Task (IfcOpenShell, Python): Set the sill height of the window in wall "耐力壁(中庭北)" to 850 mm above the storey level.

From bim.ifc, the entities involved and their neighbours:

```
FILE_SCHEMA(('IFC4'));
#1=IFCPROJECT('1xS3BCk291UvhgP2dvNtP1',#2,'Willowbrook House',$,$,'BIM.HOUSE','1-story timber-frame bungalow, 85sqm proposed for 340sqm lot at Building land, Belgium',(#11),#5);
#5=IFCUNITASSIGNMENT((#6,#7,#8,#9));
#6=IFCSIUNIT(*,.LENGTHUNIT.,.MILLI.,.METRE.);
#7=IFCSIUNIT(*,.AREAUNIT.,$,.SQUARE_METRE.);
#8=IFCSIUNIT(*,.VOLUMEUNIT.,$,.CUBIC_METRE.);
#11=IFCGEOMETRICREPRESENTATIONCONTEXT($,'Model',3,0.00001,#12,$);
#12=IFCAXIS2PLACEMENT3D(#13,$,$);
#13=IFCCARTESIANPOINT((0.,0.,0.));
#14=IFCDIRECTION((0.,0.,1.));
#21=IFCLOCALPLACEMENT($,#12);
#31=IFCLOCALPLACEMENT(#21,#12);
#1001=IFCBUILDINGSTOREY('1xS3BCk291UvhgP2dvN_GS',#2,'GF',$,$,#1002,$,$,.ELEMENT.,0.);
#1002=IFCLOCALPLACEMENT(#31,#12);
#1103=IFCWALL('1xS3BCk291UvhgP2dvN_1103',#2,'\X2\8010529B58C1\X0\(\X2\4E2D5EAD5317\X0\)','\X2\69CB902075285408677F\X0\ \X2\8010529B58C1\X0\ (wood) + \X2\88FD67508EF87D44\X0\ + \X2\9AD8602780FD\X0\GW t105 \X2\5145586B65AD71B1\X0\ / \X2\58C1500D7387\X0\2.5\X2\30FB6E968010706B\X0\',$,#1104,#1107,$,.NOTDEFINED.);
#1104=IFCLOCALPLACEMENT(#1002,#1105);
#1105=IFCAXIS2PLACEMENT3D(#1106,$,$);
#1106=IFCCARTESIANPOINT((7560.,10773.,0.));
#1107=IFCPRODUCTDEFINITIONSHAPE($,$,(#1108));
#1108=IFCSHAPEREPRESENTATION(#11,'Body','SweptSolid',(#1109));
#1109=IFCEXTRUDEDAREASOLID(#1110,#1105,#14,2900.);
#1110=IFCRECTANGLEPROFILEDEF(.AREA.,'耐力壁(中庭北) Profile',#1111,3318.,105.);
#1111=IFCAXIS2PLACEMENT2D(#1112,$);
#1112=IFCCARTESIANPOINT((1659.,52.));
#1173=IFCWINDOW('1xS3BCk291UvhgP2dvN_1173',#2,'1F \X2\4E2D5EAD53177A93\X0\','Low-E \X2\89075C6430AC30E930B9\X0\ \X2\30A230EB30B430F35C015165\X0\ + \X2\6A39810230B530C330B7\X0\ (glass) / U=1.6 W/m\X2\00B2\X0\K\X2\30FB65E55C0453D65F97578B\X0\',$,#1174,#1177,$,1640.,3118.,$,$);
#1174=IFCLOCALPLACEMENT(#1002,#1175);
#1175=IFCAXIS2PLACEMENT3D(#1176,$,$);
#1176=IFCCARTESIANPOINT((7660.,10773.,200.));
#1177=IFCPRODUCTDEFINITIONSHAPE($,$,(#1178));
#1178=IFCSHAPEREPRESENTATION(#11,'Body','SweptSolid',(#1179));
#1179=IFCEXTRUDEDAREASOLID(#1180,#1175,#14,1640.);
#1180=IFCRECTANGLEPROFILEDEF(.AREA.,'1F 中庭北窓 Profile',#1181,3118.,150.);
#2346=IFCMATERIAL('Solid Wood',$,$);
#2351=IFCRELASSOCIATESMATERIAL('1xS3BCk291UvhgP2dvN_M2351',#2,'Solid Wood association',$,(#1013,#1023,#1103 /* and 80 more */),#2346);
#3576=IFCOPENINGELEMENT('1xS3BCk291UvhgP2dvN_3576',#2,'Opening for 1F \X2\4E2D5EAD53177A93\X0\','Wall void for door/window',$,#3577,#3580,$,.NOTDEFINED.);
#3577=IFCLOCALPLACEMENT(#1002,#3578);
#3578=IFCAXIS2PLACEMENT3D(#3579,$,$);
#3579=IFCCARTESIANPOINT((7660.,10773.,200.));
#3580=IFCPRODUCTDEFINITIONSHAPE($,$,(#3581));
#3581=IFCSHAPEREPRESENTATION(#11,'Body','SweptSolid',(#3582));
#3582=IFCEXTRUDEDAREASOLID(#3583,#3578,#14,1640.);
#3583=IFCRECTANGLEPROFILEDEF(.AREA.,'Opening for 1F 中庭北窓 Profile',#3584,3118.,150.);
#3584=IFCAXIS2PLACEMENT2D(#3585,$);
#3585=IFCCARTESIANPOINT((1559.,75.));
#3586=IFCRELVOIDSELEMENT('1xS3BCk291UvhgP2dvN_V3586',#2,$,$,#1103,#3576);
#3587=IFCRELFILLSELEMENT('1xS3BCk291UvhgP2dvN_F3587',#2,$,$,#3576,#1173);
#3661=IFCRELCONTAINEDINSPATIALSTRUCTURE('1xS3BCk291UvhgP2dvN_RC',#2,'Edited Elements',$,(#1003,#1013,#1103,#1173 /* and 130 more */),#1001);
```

```python
import numpy as np
import ifcopenshell
import ifcopenshell.api.geometry
import ifcopenshell.geom
import ifcopenshell.util.element
import ifcopenshell.util.placement
import ifcopenshell.util.shape
import ifcopenshell.util.unit

model = ifcopenshell.open("bim.ifc")
unit_scale = ifcopenshell.util.unit.calculate_unit_scale(model)

window = model.by_guid("1xS3BCk291UvhgP2dvN_1173")
opening = window.FillsVoids[0].RelatingOpeningElement
storey = ifcopenshell.util.element.get_container(window, ifc_class="IfcBuildingStorey")
level = ifcopenshell.util.placement.get_local_placement(storey.ObjectPlacement)[2, 3]

# The opening's origin need not be at the sill, so measure its lowest point.
shape = ifcopenshell.geom.create_shape(ifcopenshell.geom.settings(), opening)
bottom = ifcopenshell.util.shape.get_shape_bottom_elevation(shape, shape.geometry) / unit_scale
dz = level + 850.0 - bottom

shift = np.array([0.0, 0.0, dz])
# The window is not placed relative to its opening, so move both.
for product in (opening, window):
    matrix = ifcopenshell.util.placement.get_local_placement(product.ObjectPlacement)
    matrix[:3, 3] += shift
    ifcopenshell.api.geometry.edit_object_placement(model, product=product, matrix=matrix, is_si=False)

print(f"moved by {dz * unit_scale:+.3f} m")

model.write("bim-out.ifc")
```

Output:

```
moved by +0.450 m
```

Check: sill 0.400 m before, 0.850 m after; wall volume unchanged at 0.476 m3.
